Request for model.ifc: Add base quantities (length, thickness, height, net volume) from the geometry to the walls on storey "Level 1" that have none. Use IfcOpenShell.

First a look at what the model holds.

```python
import ifcopenshell
import ifcopenshell.util.element
import ifcopenshell.util.unit

model = ifcopenshell.open("model.ifc")
print(model.schema)
for unit_type in ("LENGTHUNIT", "AREAUNIT", "VOLUMEUNIT"):
    print(unit_type, ifcopenshell.util.unit.calculate_unit_scale(model, unit_type))
storey = next(s for s in model.by_type("IfcBuildingStorey") if s.Name == "Level 1")
walls = [e for e in ifcopenshell.util.element.get_decomposition(storey) if e.is_a("IfcWall")]
for e in sorted(walls, key=lambda e: e.id()):
    print(e.id(), e.is_a(), e.Name, list(ifcopenshell.util.element.get_psets(e, qtos_only=True)), sep=" | ")
```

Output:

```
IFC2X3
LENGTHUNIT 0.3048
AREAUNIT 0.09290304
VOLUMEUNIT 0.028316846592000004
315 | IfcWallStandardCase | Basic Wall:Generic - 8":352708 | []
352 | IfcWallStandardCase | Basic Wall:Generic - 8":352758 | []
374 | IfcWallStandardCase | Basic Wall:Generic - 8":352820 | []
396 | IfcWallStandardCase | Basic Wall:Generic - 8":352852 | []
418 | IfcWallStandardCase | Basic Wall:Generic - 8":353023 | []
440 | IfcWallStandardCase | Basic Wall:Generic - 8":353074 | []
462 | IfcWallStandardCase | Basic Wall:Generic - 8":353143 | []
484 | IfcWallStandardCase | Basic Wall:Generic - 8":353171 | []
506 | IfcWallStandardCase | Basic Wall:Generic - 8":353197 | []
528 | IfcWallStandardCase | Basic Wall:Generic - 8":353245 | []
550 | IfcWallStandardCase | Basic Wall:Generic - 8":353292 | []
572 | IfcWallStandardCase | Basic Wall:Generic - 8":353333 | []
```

```python
import ifcopenshell
import ifcopenshell.api.pset
import ifcopenshell.geom
import ifcopenshell.util.element
import ifcopenshell.util.shape
import ifcopenshell.util.unit

model = ifcopenshell.open("model.ifc")
unit_scale = ifcopenshell.util.unit.calculate_unit_scale(model)
volume_scale = ifcopenshell.util.unit.calculate_unit_scale(model, "VOLUMEUNIT")
settings = ifcopenshell.geom.settings()

storey = next(s for s in model.by_type("IfcBuildingStorey") if s.Name == "Level 1")
walls = [e for e in ifcopenshell.util.element.get_decomposition(storey) if e.is_a("IfcWall")]

for e in sorted(walls, key=lambda e: e.id()):
    if ifcopenshell.util.element.get_psets(e, qtos_only=True, should_inherit=False):
        continue
    # Geometry comes back in metres, in the element's own axes.
    shape = ifcopenshell.geom.create_shape(settings, e)
    values = {
        "Length": ifcopenshell.util.shape.get_x(shape.geometry) / unit_scale,
        "Width": ifcopenshell.util.shape.get_y(shape.geometry) / unit_scale,
        "Height": ifcopenshell.util.shape.get_z(shape.geometry) / unit_scale,
        "NetVolume": ifcopenshell.util.shape.get_volume(shape.geometry) / volume_scale,
    }
    qto = ifcopenshell.api.pset.add_qto(model, product=e, name="BaseQuantities")
    ifcopenshell.api.pset.edit_qto(model, qto=qto, properties=values)
    print(e.id(), {k: round(v, 3) for k, v in values.items()})

model.write("model_v2.ifc")
```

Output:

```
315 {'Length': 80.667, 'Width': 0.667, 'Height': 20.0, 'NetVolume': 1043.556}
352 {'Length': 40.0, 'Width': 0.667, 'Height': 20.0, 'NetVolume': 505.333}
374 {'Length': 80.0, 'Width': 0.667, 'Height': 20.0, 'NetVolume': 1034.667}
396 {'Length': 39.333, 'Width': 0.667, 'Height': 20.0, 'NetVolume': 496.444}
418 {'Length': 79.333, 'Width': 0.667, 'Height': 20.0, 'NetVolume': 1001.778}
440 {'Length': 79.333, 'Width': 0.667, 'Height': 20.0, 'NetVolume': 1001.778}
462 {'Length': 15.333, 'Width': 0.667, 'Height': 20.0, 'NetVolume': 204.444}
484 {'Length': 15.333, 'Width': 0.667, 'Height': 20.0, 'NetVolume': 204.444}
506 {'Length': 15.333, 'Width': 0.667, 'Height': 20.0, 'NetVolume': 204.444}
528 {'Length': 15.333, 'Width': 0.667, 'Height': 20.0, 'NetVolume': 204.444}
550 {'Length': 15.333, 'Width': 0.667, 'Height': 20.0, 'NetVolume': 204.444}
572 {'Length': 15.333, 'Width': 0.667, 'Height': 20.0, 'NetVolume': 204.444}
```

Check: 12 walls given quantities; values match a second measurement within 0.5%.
